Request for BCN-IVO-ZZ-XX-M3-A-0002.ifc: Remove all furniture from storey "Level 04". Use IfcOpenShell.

First a look at what the model holds.

```python
import ifcopenshell
import ifcopenshell.util.element

model = ifcopenshell.open("BCN-IVO-ZZ-XX-M3-A-0002.ifc")
print(model.schema)
storey = next(s for s in model.by_type("IfcBuildingStorey") if s.Name == "Level 04")
furniture = [e for e in ifcopenshell.util.element.get_decomposition(storey) if e.is_a("IfcFurnishingElement")]
seen = {}
for e in furniture:
    element_type = ifcopenshell.util.element.get_type(e)
    name = element_type.Name if element_type not in (None, e) else None
    seen[name] = seen.get(name, 0) + 1
for name, count in sorted(seen.items(), key=str):
    print(count, "x", name)
```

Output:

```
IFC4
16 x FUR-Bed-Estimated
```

```python
import ifcopenshell
import ifcopenshell.api.root
import ifcopenshell.util.element

model = ifcopenshell.open("BCN-IVO-ZZ-XX-M3-A-0002.ifc")

storey = next(s for s in model.by_type("IfcBuildingStorey") if s.Name == "Level 04")
furniture = [e for e in ifcopenshell.util.element.get_decomposition(storey) if e.is_a("IfcFurnishingElement")]

for e in furniture:
    ifcopenshell.api.root.remove_product(model, product=e)
print(len(furniture), "removed")

model.write("BCN-IVO-ZZ-XX-M3-A-0002_updated.ifc")
```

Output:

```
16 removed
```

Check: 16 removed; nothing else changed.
